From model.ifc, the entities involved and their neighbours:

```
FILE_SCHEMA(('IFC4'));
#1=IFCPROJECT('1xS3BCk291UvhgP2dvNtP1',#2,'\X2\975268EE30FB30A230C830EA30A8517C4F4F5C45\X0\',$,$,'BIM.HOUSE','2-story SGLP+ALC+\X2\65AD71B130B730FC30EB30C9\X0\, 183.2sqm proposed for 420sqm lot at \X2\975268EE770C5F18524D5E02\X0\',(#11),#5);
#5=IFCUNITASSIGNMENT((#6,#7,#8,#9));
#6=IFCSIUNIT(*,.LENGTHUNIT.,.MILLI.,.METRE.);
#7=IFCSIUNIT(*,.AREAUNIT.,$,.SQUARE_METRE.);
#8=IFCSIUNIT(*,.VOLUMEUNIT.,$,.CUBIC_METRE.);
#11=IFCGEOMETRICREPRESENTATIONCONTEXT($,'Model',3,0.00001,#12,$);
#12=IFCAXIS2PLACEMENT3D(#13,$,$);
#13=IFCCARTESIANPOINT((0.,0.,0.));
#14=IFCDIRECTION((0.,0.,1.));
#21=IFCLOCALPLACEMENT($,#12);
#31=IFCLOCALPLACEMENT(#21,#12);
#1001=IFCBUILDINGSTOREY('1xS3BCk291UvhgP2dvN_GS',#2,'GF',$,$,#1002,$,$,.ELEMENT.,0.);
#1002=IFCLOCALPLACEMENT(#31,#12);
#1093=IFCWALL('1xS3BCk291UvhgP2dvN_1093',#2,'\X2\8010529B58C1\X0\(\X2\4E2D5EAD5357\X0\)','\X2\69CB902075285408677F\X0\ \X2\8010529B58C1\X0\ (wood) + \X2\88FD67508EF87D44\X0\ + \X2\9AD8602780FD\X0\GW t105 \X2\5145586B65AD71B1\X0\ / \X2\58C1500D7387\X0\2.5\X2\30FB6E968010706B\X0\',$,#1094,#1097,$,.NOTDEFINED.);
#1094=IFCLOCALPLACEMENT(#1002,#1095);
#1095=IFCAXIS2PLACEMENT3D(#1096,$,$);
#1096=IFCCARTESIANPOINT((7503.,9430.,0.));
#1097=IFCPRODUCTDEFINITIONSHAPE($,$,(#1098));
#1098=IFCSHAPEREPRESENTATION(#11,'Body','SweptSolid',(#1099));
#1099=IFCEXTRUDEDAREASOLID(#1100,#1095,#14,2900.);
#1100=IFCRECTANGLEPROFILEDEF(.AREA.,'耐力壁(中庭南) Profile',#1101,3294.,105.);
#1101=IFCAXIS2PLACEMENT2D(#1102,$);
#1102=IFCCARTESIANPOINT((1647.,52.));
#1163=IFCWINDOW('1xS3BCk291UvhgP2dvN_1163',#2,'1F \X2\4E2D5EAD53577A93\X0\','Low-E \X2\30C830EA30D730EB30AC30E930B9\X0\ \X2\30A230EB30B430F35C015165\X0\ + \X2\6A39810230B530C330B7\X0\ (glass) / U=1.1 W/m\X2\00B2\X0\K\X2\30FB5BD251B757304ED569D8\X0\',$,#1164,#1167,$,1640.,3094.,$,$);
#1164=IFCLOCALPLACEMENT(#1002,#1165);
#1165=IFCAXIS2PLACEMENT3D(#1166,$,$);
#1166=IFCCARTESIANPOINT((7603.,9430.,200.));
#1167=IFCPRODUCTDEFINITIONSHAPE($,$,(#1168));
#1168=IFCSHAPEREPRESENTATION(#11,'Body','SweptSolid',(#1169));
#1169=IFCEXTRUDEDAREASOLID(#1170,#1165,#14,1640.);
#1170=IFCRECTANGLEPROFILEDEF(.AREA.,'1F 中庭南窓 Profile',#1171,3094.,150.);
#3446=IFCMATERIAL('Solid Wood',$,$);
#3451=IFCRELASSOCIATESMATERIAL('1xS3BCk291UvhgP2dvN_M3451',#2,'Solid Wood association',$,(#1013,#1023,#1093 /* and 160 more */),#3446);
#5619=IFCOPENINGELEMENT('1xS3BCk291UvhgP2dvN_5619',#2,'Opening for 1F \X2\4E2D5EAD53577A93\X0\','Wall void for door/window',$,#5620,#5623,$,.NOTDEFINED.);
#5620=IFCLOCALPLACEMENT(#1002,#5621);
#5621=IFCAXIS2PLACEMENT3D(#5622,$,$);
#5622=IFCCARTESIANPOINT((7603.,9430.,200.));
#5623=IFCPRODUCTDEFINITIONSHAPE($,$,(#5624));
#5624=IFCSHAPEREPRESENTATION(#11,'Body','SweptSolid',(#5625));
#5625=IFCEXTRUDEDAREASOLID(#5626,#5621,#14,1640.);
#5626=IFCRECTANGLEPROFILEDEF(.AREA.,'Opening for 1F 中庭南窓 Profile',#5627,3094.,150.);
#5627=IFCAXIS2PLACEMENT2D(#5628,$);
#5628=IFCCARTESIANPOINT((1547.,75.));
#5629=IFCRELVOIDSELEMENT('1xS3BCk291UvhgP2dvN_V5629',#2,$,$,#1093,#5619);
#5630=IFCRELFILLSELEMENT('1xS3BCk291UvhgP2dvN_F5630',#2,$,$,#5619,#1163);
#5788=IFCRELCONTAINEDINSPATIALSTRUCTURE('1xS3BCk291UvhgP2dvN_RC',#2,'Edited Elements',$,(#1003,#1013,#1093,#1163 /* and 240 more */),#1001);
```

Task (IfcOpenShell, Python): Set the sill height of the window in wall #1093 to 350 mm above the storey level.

```python
import numpy as np
import ifcopenshell
import ifcopenshell.api.geometry
import ifcopenshell.geom
import ifcopenshell.util.element
import ifcopenshell.util.placement
import ifcopenshell.util.shape
import ifcopenshell.util.unit

model = ifcopenshell.open("model.ifc")
unit_scale = ifcopenshell.util.unit.calculate_unit_scale(model)

window = model.by_guid("1xS3BCk291UvhgP2dvN_1163")
opening = window.FillsVoids[0].RelatingOpeningElement
storey = ifcopenshell.util.element.get_container(window, ifc_class="IfcBuildingStorey")
level = ifcopenshell.util.placement.get_local_placement(storey.ObjectPlacement)[2, 3]

# The opening's origin need not be at the sill, so measure its lowest point.
shape = ifcopenshell.geom.create_shape(ifcopenshell.geom.settings(), opening)
bottom = ifcopenshell.util.shape.get_shape_bottom_elevation(shape, shape.geometry) / unit_scale
dz = level + 0.35 / unit_scale - bottom

shift = np.array([0.0, 0.0, dz])
# The window is not placed relative to its opening, so move both.
for product in (opening, window):
    matrix = ifcopenshell.util.placement.get_local_placement(product.ObjectPlacement)
    matrix[:3, 3] += shift
    ifcopenshell.api.geometry.edit_object_placement(model, product=product, matrix=matrix, is_si=False)

print(f"moved by {dz * unit_scale:+.3f} m")

model.write("model_updated.ifc")
```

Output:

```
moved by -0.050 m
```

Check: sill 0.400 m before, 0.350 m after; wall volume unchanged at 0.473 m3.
